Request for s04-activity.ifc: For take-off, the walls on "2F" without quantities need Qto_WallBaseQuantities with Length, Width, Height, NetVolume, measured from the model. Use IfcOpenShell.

First a look at what the model holds.

```python
import ifcopenshell
import ifcopenshell.util.element
import ifcopenshell.util.unit

model = ifcopenshell.open("s04-activity.ifc")
print(model.schema)
for unit_type in ("LENGTHUNIT", "AREAUNIT", "VOLUMEUNIT"):
    print(unit_type, ifcopenshell.util.unit.calculate_unit_scale(model, unit_type))
storey = next(s for s in model.by_type("IfcBuildingStorey") if s.Name == "2F")
walls = [e for e in ifcopenshell.util.element.get_decomposition(storey) if e.is_a("IfcWall")]
for e in sorted(walls, key=lambda e: e.id()):
    print(e.id(), e.is_a(), e.Name, list(ifcopenshell.util.element.get_psets(e, qtos_only=True)), sep=" | ")
```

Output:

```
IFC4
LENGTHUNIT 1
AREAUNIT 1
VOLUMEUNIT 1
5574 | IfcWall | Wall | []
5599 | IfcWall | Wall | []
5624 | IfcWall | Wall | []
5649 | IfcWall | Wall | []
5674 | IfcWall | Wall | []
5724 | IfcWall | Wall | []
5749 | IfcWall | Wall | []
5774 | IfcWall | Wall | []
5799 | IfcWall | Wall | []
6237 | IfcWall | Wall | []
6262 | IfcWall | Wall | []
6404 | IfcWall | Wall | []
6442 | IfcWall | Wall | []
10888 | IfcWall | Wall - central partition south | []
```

```python
import ifcopenshell
import ifcopenshell.api.pset
import ifcopenshell.geom
import ifcopenshell.util.element
import ifcopenshell.util.shape
import ifcopenshell.util.unit

model = ifcopenshell.open("s04-activity.ifc")
unit_scale = ifcopenshell.util.unit.calculate_unit_scale(model)
volume_scale = ifcopenshell.util.unit.calculate_unit_scale(model, "VOLUMEUNIT")
settings = ifcopenshell.geom.settings()

storey = next(s for s in model.by_type("IfcBuildingStorey") if s.Name == "2F")
walls = [e for e in ifcopenshell.util.element.get_decomposition(storey) if e.is_a("IfcWall")]

for e in sorted(walls, key=lambda e: e.id()):
    if ifcopenshell.util.element.get_psets(e, qtos_only=True, should_inherit=False):
        continue
    # Geometry comes back in metres, in the element's own axes.
    shape = ifcopenshell.geom.create_shape(settings, e)
    values = {
        "Length": ifcopenshell.util.shape.get_x(shape.geometry) / unit_scale,
        "Width": ifcopenshell.util.shape.get_y(shape.geometry) / unit_scale,
        "Height": ifcopenshell.util.shape.get_z(shape.geometry) / unit_scale,
        "NetVolume": ifcopenshell.util.shape.get_volume(shape.geometry) / volume_scale,
    }
    qto = ifcopenshell.api.pset.add_qto(model, product=e, name="Qto_WallBaseQuantities")
    ifcopenshell.api.pset.edit_qto(model, qto=qto, properties=values)
    print(e.id(), {k: round(v, 3) for k, v in values.items()})

model.write("s04-activity_edited.ifc")
```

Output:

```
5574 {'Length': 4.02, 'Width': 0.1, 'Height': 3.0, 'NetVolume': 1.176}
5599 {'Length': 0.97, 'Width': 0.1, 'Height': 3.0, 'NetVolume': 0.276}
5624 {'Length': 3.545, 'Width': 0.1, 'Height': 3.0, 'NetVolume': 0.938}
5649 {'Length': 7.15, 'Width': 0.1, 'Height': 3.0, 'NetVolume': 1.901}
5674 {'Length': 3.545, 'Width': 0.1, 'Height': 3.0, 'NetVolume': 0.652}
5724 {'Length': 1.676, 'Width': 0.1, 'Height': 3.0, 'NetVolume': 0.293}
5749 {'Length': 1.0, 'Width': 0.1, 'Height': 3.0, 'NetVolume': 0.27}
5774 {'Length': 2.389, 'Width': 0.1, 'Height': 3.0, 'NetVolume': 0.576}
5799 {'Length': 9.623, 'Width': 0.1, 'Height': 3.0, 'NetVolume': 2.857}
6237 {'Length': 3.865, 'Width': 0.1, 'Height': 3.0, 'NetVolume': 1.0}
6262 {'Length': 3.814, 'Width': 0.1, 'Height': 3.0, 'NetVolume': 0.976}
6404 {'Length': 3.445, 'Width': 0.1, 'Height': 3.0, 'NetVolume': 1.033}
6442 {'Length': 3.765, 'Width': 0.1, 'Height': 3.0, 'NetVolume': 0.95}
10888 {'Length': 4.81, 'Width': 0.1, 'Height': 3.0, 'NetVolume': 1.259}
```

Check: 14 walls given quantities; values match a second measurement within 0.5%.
